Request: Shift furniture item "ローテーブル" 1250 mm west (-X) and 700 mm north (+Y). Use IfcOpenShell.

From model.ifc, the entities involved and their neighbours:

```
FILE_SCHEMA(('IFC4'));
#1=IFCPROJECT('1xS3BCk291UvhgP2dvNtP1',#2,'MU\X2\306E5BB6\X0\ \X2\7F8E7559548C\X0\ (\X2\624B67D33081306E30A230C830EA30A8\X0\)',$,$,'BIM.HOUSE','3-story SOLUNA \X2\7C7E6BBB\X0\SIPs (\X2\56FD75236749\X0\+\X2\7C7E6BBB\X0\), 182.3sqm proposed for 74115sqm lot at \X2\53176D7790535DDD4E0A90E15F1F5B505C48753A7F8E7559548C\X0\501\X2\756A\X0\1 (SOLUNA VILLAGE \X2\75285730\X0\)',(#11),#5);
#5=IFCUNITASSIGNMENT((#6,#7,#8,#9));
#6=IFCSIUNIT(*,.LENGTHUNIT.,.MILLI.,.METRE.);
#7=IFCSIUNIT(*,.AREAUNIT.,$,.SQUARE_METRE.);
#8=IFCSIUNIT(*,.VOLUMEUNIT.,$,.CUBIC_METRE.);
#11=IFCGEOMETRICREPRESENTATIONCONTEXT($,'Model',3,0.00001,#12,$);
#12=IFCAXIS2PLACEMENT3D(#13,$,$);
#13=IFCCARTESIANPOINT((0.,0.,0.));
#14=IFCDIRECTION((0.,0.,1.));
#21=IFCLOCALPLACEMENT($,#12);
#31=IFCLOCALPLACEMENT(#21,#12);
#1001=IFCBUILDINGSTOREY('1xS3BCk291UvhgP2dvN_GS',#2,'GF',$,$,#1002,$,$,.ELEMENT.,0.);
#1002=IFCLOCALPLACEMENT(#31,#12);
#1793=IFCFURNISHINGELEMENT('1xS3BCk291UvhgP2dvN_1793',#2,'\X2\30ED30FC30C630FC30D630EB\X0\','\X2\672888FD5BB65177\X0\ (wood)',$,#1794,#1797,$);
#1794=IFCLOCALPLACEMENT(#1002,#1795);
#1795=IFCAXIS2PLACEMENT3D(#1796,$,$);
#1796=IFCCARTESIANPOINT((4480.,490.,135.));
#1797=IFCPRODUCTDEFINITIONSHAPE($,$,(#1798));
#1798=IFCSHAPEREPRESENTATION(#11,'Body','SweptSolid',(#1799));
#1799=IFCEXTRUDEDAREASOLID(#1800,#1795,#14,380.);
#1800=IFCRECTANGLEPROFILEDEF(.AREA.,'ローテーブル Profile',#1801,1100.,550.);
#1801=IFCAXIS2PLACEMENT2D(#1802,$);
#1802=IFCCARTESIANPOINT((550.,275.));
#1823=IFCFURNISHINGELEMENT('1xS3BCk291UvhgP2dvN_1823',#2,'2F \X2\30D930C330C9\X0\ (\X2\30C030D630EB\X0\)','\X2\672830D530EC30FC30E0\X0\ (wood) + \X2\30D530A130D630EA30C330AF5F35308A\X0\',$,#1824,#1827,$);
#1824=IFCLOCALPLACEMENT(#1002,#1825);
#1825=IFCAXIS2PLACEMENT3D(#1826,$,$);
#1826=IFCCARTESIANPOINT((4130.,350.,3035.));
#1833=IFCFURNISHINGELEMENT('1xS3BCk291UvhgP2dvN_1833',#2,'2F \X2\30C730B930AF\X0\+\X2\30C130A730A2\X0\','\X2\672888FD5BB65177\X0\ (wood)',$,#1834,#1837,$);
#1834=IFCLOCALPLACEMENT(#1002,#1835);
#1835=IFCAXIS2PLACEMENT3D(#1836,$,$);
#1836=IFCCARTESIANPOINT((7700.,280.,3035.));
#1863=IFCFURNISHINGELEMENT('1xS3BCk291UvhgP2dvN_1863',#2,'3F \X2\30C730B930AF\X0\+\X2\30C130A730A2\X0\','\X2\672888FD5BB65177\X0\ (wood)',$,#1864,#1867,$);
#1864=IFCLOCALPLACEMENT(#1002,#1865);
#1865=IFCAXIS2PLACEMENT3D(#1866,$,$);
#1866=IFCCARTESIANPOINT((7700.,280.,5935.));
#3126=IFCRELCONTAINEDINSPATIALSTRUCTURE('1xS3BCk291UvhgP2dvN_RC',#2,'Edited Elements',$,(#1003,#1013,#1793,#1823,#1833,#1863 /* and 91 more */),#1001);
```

```python
import ifcopenshell
import ifcopenshell.api.geometry
import ifcopenshell.util.placement
import ifcopenshell.util.unit

model = ifcopenshell.open("model.ifc")
unit_scale = ifcopenshell.util.unit.calculate_unit_scale(model)

item = model.by_id(1793)
matrix = ifcopenshell.util.placement.get_local_placement(item.ObjectPlacement)
matrix[0, 3] -= 1.25 / unit_scale
matrix[1, 3] += 0.7 / unit_scale
ifcopenshell.api.geometry.edit_object_placement(model, product=item, matrix=matrix, is_si=False)

print(ifcopenshell.util.placement.get_local_placement(item.ObjectPlacement).round(3) + 0.0)

model.write("model_rev.ifc")
```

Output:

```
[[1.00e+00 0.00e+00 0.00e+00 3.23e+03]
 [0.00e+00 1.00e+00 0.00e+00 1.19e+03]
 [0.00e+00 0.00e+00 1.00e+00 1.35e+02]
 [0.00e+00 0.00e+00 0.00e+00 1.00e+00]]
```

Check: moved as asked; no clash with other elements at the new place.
